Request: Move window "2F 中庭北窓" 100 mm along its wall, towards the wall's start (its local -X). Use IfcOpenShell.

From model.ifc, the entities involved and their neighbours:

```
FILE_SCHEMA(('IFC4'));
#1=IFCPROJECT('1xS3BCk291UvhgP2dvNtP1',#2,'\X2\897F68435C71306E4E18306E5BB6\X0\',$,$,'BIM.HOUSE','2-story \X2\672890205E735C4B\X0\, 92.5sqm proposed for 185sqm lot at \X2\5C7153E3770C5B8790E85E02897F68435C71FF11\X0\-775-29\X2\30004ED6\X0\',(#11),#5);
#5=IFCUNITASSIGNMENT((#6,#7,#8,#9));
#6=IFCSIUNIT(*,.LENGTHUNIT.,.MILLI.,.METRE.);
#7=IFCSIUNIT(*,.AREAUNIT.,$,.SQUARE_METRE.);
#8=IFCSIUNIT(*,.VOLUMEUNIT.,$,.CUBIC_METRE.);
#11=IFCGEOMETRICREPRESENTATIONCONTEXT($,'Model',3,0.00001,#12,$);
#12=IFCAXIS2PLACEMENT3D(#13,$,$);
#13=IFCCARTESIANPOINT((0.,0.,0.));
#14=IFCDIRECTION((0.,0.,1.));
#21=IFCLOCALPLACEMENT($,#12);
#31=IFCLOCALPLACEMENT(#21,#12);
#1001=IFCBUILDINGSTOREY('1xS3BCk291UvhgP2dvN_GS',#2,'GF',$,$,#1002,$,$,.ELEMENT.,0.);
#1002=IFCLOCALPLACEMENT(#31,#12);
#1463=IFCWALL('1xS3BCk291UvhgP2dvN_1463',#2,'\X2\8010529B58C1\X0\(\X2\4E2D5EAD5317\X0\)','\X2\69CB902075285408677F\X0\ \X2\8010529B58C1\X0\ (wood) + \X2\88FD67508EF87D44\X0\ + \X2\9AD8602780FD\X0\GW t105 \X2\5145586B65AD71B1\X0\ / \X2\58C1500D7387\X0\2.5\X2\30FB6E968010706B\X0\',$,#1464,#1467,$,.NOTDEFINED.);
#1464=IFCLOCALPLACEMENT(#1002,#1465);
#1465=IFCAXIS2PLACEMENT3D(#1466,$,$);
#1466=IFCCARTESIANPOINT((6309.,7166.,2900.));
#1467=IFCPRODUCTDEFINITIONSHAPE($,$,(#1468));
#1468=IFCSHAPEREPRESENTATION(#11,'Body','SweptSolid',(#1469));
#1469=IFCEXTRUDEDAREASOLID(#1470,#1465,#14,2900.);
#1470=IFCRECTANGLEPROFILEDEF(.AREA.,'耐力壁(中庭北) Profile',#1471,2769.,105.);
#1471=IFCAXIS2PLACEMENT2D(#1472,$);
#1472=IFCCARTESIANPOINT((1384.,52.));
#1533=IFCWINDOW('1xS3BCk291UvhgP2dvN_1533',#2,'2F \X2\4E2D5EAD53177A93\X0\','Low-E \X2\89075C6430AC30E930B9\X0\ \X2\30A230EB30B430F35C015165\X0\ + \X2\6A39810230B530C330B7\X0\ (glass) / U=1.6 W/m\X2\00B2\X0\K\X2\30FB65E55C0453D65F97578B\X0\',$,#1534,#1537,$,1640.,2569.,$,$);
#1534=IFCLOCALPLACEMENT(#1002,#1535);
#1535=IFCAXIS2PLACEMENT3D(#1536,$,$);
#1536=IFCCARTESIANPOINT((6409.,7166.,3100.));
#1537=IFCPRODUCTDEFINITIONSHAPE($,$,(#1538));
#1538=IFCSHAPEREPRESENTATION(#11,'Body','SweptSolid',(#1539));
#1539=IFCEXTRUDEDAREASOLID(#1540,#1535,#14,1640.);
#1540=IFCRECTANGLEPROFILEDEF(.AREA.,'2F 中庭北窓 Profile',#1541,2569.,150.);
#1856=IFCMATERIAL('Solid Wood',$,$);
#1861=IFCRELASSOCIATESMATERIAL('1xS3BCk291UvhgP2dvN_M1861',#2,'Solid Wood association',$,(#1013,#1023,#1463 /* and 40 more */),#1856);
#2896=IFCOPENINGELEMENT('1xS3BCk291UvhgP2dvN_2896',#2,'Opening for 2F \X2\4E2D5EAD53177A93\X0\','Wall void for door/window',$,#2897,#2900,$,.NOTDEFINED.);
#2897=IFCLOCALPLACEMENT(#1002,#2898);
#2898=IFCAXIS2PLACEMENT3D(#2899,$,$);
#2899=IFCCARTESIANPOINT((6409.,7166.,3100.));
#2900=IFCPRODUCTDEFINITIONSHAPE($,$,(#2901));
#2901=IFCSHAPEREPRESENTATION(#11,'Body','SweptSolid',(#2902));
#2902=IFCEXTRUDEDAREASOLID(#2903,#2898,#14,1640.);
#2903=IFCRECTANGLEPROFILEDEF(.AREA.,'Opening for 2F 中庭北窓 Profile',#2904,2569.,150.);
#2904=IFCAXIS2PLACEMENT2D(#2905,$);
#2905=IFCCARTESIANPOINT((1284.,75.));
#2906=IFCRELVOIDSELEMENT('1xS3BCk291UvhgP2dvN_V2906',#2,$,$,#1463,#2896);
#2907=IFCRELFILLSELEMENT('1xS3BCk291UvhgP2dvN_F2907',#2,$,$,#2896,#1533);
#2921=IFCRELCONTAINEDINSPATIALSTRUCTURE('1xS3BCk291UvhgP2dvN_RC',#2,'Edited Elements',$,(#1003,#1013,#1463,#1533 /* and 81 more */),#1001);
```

```python
import ifcopenshell
import ifcopenshell.api.geometry
import ifcopenshell.util.placement
import ifcopenshell.util.unit

model = ifcopenshell.open("model.ifc")
unit_scale = ifcopenshell.util.unit.calculate_unit_scale(model)

window = model.by_guid("1xS3BCk291UvhgP2dvN_1533")
opening = window.FillsVoids[0].RelatingOpeningElement
wall = opening.VoidsElements[0].RelatingBuildingElement

wall_matrix = ifcopenshell.util.placement.get_local_placement(wall.ObjectPlacement)
shift = wall_matrix[:3, 0] * -0.1 / unit_scale
before = ifcopenshell.util.placement.get_local_placement(window.ObjectPlacement)[:3, 3].copy()

# The window is not placed relative to its opening, so move both.
for product in (opening, window):
    matrix = ifcopenshell.util.placement.get_local_placement(product.ObjectPlacement)
    matrix[:3, 3] += shift
    ifcopenshell.api.geometry.edit_object_placement(model, product=product, matrix=matrix, is_si=False)

after = ifcopenshell.util.placement.get_local_placement(window.ObjectPlacement)[:3, 3]
print("window moved by", (after - before).round(3) + 0.0)

model.write("model_v2.ifc")
```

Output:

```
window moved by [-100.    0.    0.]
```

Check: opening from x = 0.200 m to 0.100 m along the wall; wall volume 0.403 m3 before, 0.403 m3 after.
